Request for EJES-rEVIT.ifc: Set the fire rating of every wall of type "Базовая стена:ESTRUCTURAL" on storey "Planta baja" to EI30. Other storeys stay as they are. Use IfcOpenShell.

First a look at what the model holds.

```python
import ifcopenshell
import ifcopenshell.util.element

model = ifcopenshell.open("EJES-rEVIT.ifc")
print(model.schema)
storey = next(s for s in model.by_type("IfcBuildingStorey") if s.Name == "Planta baja")
walls = [e for e in ifcopenshell.util.element.get_decomposition(storey) if e.is_a("IfcWall")]
seen = {}
for e in walls:
    element_type = ifcopenshell.util.element.get_type(e)
    key = (element_type.Name if element_type != e and element_type else None, ifcopenshell.util.element.get_pset(e, "Pset_WallCommon", "FireRating"))
    seen[key] = seen.get(key, 0) + 1
for (name, value), count in sorted(seen.items(), key=str):
    print(count, "x", name, "|", value)
```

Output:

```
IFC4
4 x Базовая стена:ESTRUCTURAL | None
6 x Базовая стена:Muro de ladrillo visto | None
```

```python
import ifcopenshell
import ifcopenshell.api.pset
import ifcopenshell.util.element

model = ifcopenshell.open("EJES-rEVIT.ifc")

storey = next(s for s in model.by_type("IfcBuildingStorey") if s.Name == "Planta baja")
walls = [e for e in ifcopenshell.util.element.get_decomposition(storey) if e.is_a("IfcWall")]

count = 0
for e in walls:
    element_type = ifcopenshell.util.element.get_type(e)
    if element_type in (None, e) or element_type.Name != "Базовая стена:ESTRUCTURAL":
        continue
    # add_pset returns the element's existing set when there is one.
    pset = ifcopenshell.api.pset.add_pset(model, product=e, name="Pset_WallCommon")
    ifcopenshell.api.pset.edit_pset(model, pset=pset, properties={"FireRating": "EI30"})
    count += 1

print(count, "walls updated")

model.write("EJES-rEVIT_v2.ifc")
```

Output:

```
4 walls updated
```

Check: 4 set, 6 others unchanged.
